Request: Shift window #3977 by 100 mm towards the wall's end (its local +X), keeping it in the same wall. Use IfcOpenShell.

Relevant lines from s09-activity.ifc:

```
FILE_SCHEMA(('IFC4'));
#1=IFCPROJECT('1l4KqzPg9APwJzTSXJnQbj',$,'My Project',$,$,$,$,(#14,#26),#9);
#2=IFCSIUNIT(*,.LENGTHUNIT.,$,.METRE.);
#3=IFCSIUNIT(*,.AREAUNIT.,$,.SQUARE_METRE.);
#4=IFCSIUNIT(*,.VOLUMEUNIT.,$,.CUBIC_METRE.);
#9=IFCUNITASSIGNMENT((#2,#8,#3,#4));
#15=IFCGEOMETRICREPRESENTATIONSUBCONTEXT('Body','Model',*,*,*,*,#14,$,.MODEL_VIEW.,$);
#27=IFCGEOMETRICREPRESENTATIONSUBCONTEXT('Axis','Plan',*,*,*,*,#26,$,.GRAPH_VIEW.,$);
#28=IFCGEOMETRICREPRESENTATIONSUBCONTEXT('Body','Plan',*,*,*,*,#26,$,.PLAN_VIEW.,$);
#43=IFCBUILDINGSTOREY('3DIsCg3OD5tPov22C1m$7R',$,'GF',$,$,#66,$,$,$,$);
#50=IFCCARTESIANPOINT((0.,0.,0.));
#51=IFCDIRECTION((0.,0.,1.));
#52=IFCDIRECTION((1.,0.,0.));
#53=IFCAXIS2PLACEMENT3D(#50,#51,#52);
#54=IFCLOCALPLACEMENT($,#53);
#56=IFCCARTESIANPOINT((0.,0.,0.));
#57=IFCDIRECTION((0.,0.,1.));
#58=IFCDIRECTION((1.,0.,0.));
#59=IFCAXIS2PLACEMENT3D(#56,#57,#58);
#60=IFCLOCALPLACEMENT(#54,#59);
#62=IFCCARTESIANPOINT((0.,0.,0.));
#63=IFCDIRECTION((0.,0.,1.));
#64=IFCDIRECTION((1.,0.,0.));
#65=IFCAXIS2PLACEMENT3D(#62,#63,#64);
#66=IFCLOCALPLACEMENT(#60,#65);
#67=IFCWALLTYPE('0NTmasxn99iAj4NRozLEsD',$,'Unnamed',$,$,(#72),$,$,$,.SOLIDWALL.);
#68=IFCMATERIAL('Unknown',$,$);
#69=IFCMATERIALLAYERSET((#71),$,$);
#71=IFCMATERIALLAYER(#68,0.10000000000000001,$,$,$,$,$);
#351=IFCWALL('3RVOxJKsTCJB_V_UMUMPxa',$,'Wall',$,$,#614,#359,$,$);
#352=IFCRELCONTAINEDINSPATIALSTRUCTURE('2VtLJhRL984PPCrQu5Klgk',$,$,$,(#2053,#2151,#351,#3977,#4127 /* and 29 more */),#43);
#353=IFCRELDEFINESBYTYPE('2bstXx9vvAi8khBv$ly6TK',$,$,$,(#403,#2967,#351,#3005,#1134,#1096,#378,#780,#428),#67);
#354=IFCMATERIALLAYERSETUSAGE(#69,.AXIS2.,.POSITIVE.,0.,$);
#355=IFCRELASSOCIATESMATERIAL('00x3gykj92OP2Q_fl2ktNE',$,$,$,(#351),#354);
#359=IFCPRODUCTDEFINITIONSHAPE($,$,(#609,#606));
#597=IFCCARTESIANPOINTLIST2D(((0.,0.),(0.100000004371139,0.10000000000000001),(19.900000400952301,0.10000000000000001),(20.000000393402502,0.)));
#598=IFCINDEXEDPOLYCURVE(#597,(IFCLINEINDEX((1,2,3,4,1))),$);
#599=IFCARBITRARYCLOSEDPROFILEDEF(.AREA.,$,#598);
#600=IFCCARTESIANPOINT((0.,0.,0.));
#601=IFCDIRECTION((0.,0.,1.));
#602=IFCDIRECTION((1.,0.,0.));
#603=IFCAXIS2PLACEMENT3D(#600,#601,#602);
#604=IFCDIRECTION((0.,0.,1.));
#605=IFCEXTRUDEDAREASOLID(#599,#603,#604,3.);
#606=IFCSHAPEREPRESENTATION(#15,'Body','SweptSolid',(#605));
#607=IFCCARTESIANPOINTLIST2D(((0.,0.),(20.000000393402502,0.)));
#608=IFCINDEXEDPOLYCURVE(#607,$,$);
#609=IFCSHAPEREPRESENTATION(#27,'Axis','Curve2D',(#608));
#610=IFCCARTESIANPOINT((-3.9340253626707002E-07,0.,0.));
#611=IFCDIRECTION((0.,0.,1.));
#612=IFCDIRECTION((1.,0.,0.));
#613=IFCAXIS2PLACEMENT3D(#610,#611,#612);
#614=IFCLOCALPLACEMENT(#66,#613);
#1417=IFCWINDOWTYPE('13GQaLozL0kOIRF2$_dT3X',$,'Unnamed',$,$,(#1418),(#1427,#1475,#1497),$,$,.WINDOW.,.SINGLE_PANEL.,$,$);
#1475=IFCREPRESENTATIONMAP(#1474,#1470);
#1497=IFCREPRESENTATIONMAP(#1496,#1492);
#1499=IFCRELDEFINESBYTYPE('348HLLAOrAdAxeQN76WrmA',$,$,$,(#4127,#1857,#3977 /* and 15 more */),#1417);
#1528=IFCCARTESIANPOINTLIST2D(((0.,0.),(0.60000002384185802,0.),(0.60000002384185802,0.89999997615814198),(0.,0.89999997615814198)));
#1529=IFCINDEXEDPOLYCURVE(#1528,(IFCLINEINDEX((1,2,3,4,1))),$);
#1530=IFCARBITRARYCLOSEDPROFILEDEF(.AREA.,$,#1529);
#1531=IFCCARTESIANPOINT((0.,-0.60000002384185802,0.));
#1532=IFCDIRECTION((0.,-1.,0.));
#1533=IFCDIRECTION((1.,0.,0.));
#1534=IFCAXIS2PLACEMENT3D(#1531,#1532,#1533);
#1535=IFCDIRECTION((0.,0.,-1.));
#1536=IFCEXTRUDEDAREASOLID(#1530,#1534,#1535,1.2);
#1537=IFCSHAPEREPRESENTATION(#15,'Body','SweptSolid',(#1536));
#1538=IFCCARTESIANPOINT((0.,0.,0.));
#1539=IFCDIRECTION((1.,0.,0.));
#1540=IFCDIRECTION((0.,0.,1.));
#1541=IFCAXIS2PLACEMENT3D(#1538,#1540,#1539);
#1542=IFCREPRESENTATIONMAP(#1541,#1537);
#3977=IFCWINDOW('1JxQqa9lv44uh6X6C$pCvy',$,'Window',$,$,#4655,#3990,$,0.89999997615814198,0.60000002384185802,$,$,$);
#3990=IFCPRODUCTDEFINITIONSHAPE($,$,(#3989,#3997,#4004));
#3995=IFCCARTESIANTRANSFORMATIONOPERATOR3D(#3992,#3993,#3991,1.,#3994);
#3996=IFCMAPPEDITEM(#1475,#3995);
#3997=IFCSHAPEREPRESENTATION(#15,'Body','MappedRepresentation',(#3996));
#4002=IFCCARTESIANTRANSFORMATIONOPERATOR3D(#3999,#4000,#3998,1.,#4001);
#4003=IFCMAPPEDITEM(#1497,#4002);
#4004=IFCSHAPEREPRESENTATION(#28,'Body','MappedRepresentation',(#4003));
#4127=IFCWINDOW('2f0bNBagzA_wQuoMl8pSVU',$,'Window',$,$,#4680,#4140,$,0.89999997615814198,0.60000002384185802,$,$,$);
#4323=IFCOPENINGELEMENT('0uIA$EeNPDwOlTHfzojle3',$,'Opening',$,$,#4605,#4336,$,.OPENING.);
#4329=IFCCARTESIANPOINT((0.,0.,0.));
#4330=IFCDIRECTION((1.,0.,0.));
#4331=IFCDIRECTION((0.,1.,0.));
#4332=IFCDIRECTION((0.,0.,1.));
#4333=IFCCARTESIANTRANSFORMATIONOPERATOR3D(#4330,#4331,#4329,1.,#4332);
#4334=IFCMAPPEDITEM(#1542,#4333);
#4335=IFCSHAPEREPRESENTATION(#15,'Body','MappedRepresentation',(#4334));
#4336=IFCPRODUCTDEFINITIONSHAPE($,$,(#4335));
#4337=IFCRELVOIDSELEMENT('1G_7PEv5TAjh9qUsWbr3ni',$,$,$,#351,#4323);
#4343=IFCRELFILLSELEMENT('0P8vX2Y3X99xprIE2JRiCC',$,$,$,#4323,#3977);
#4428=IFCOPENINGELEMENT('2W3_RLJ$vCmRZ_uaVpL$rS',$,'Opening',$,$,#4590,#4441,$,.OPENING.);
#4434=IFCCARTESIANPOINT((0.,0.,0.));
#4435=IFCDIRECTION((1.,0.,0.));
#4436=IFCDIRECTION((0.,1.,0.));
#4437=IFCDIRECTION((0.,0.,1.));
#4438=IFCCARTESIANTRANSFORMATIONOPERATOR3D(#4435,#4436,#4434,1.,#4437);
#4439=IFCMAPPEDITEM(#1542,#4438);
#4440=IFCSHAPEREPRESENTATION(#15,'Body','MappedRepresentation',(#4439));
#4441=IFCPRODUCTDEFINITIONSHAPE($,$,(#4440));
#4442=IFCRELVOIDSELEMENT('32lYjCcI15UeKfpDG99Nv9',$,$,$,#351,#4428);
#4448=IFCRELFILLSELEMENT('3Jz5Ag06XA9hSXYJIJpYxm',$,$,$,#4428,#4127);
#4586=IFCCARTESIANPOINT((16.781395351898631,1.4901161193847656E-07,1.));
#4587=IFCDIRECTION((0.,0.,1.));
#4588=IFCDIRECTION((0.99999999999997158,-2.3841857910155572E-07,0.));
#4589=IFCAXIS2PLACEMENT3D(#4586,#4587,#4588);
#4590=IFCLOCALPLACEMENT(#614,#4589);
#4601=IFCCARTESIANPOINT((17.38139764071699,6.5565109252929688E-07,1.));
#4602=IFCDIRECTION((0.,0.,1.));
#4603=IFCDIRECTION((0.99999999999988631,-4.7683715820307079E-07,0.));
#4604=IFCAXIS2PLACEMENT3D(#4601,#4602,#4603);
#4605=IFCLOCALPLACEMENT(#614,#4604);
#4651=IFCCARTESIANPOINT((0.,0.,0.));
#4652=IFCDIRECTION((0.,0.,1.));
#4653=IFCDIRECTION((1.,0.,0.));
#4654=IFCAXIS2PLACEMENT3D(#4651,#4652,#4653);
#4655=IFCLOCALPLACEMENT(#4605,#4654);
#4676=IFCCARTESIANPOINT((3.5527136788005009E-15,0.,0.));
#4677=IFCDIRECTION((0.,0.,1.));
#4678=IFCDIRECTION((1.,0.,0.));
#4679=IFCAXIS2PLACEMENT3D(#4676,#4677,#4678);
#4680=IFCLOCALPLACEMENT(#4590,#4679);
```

```python
import ifcopenshell
import ifcopenshell.api.geometry
import ifcopenshell.util.placement
import ifcopenshell.util.unit

model = ifcopenshell.open("s09-activity.ifc")
unit_scale = ifcopenshell.util.unit.calculate_unit_scale(model)

window = model.by_guid("1JxQqa9lv44uh6X6C$pCvy")
opening = window.FillsVoids[0].RelatingOpeningElement
wall = opening.VoidsElements[0].RelatingBuildingElement

wall_matrix = ifcopenshell.util.placement.get_local_placement(wall.ObjectPlacement)
shift = wall_matrix[:3, 0] * 0.1 / unit_scale
before = ifcopenshell.util.placement.get_local_placement(window.ObjectPlacement)[:3, 3].copy()

# The window is placed relative to its opening, so it follows when the opening moves.
matrix = ifcopenshell.util.placement.get_local_placement(opening.ObjectPlacement)
matrix[:3, 3] += shift
ifcopenshell.api.geometry.edit_object_placement(
    model, product=opening, matrix=matrix, is_si=False, should_transform_children=True
)

after = ifcopenshell.util.placement.get_local_placement(window.ObjectPlacement)[:3, 3]
print("window moved by", (after - before).round(3) + 0.0)

model.write("s09-activity_edited.ifc")
```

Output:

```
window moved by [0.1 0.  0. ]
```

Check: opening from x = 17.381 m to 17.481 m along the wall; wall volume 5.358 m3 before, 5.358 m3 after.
